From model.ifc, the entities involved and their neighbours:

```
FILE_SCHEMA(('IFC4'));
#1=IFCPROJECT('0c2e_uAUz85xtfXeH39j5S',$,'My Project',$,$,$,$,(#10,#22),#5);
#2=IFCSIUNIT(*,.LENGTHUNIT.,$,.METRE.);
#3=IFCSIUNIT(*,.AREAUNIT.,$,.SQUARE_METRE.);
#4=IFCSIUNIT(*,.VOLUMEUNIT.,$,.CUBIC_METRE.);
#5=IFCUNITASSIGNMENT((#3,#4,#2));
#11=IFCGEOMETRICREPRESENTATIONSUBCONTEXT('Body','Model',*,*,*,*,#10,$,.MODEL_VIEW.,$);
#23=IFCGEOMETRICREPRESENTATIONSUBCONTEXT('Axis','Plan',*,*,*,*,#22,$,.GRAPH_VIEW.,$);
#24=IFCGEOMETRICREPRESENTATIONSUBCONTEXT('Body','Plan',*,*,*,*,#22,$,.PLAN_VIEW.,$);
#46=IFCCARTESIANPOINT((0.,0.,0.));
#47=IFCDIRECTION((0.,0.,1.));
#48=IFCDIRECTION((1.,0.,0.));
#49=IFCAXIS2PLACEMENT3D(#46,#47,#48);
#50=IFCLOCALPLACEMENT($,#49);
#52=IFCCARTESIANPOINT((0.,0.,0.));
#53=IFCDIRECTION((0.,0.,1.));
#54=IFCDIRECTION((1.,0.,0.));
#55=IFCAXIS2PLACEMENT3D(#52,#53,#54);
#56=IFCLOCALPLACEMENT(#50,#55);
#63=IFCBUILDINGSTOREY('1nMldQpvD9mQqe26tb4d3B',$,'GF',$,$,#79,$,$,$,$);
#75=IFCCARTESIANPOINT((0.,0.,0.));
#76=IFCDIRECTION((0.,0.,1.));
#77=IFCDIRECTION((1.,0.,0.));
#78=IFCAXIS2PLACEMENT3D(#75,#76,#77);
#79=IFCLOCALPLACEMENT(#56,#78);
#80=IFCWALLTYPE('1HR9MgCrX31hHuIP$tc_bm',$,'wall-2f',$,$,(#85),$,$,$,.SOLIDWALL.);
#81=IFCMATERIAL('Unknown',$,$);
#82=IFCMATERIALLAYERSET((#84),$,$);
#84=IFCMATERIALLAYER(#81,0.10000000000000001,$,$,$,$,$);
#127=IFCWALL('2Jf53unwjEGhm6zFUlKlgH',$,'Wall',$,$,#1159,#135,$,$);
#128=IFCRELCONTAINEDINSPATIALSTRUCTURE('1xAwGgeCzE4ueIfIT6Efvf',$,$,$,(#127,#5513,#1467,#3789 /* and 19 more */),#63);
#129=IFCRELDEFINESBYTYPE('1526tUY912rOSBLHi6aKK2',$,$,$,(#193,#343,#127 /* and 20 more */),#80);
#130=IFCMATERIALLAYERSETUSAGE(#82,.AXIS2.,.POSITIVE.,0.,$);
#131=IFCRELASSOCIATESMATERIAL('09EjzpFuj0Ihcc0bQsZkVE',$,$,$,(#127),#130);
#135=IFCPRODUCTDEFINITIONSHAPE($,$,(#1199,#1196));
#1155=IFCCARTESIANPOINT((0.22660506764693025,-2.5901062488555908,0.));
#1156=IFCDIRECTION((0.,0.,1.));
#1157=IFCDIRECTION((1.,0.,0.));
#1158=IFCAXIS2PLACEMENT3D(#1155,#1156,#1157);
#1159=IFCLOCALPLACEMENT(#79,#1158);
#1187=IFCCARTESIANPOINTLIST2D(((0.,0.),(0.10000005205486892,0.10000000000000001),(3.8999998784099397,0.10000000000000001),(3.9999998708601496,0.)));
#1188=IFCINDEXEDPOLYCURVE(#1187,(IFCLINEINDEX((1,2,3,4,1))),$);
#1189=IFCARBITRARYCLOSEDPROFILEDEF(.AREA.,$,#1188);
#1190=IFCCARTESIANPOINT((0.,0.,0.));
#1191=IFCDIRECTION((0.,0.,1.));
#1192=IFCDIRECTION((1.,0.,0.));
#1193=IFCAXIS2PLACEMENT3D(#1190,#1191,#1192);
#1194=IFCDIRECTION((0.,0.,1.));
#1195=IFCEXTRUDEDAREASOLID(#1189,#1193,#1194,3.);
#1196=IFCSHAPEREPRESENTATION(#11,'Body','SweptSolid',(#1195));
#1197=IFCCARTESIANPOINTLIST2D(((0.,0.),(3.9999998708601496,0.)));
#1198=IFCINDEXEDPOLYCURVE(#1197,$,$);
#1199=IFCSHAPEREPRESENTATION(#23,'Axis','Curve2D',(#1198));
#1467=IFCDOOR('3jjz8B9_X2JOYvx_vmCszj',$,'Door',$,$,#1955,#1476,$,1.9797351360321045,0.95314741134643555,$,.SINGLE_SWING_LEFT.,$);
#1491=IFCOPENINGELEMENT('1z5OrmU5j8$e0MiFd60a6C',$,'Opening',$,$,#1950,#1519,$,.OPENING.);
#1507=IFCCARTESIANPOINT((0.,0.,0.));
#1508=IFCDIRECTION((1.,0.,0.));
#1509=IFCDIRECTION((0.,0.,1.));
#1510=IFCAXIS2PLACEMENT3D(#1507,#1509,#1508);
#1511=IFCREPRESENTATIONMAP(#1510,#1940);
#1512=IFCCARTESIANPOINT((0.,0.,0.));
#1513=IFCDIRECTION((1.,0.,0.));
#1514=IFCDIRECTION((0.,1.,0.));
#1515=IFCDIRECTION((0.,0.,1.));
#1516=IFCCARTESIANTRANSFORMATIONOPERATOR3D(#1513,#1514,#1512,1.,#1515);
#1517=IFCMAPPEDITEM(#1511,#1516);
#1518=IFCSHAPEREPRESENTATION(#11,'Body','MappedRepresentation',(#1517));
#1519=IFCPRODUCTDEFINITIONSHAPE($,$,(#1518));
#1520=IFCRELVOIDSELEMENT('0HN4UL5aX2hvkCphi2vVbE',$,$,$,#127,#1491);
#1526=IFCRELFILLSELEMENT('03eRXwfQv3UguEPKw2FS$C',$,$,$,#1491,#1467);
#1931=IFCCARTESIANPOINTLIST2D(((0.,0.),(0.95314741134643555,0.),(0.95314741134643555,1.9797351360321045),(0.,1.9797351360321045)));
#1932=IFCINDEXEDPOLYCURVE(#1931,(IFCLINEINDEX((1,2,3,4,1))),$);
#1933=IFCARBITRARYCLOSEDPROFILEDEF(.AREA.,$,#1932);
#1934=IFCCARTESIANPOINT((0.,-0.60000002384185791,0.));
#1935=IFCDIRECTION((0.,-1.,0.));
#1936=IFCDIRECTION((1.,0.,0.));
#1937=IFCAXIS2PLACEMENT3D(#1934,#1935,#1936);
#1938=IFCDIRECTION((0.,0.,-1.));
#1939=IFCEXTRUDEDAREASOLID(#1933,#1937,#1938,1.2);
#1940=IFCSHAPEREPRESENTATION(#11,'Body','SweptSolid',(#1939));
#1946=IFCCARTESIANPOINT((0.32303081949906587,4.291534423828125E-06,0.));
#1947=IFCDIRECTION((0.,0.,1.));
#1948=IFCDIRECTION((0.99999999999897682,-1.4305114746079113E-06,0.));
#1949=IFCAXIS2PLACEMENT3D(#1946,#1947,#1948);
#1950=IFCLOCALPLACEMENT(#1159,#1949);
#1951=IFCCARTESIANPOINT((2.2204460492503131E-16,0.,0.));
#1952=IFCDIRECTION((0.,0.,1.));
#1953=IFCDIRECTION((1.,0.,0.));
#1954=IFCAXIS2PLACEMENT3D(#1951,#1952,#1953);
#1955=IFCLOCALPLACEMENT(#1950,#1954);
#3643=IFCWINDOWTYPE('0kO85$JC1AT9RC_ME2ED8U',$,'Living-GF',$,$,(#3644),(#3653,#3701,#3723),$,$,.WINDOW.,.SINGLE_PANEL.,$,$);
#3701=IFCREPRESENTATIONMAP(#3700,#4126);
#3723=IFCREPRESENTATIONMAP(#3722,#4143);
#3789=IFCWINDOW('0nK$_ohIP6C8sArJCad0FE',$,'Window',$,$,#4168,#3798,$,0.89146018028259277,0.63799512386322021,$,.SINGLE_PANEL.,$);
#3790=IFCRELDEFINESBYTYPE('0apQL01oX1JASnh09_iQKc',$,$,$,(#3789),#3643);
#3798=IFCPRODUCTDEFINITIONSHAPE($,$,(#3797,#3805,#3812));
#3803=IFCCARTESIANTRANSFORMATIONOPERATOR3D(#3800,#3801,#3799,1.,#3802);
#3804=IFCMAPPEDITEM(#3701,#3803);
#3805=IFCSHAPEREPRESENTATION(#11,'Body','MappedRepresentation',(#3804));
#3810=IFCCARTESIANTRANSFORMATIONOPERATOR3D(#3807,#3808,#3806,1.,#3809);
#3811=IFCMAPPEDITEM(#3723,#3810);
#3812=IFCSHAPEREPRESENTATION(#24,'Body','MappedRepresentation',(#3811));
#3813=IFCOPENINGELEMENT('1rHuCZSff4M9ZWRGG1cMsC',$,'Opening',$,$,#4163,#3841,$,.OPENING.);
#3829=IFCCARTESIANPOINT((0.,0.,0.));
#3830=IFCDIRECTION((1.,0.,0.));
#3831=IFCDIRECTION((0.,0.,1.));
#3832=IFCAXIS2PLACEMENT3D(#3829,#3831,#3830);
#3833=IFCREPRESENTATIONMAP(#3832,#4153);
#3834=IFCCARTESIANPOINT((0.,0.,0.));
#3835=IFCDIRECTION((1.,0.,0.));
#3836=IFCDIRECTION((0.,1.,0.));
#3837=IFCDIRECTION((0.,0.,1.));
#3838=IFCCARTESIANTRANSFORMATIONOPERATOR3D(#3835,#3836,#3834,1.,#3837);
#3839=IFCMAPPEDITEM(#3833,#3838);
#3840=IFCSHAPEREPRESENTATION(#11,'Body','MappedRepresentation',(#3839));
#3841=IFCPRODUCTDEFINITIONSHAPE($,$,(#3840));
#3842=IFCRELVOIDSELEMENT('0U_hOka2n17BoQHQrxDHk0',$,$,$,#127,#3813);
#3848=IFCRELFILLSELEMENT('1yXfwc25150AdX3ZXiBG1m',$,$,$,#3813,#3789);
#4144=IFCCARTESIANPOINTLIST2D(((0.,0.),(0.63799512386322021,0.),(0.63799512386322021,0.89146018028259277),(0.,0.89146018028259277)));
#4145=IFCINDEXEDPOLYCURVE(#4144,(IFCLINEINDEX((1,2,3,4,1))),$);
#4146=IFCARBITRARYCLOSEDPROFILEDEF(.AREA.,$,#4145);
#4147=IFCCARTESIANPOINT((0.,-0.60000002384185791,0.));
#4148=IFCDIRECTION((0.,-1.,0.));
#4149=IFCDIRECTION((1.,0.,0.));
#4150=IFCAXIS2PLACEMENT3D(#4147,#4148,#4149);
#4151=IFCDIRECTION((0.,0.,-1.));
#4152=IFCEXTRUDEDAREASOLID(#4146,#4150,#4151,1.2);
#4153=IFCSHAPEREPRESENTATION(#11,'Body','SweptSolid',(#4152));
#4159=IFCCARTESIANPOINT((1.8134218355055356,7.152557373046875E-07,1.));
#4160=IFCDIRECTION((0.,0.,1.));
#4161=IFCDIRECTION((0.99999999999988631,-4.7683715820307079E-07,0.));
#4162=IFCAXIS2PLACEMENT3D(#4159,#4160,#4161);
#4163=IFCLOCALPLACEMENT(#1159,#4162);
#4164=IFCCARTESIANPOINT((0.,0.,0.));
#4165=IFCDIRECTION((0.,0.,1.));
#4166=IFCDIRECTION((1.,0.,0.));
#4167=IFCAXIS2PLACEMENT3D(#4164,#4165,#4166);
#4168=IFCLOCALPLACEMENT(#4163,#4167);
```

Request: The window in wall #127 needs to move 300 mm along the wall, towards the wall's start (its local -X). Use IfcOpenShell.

```python
import ifcopenshell
import ifcopenshell.api.geometry
import ifcopenshell.util.placement
import ifcopenshell.util.unit

model = ifcopenshell.open("model.ifc")
unit_scale = ifcopenshell.util.unit.calculate_unit_scale(model)

window = model.by_id(3789)
opening = window.FillsVoids[0].RelatingOpeningElement
wall = opening.VoidsElements[0].RelatingBuildingElement

wall_matrix = ifcopenshell.util.placement.get_local_placement(wall.ObjectPlacement)
shift = wall_matrix[:3, 0] * -0.3 / unit_scale
before = ifcopenshell.util.placement.get_local_placement(window.ObjectPlacement)[:3, 3].copy()

# The window is placed relative to its opening, so it follows when the opening moves.
matrix = ifcopenshell.util.placement.get_local_placement(opening.ObjectPlacement)
matrix[:3, 3] += shift
ifcopenshell.api.geometry.edit_object_placement(
    model, product=opening, matrix=matrix, is_si=False, should_transform_children=True
)

after = ifcopenshell.util.placement.get_local_placement(window.ObjectPlacement)[:3, 3]
print("window moved by", (after - before).round(3) + 0.0)

model.write("model_rev.ifc")
```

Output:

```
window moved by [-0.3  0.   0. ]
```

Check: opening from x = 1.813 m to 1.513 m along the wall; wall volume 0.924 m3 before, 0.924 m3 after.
